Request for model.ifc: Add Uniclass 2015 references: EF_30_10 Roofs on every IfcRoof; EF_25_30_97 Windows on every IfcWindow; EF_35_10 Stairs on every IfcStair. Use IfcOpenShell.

First a look at what the model holds.

```python
import ifcopenshell

model = ifcopenshell.open("model.ifc")
print(model.schema)
print("classifications:", [c.Name for c in model.by_type("IfcClassification")])
for ifc_class in ("IfcDoor", "IfcRoof", "IfcStair", "IfcWall", "IfcWindow"):
    print(ifc_class, len(model.by_type(ifc_class)))
```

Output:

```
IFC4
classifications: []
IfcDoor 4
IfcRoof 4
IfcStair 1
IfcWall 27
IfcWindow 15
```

```python
import ifcopenshell
import ifcopenshell.api.classification

model = ifcopenshell.open("model.ifc")

system = ifcopenshell.api.classification.add_classification(model, classification="Uniclass 2015")

codes = {
    "IfcRoof": ("EF_30_10", "Roofs"),
    "IfcWindow": ("EF_25_30_97", "Windows"),
    "IfcStair": ("EF_35_10", "Stairs"),
}
for ifc_class, (code, name) in codes.items():
    products = model.by_type(ifc_class)
    ifcopenshell.api.classification.add_reference(
        model, products=products, classification=system, identification=code, name=name
    )
    print(code, len(products))

model.write("model-out.ifc")
```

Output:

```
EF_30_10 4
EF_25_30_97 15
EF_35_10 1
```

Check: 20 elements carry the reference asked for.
